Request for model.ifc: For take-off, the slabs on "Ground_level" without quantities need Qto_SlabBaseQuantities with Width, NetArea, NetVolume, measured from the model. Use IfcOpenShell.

First a look at what the model holds.

```python
import ifcopenshell
import ifcopenshell.util.element
import ifcopenshell.util.unit

model = ifcopenshell.open("model.ifc")
print(model.schema)
for unit_type in ("LENGTHUNIT", "AREAUNIT", "VOLUMEUNIT"):
    print(unit_type, ifcopenshell.util.unit.calculate_unit_scale(model, unit_type))
storey = next(s for s in model.by_type("IfcBuildingStorey") if s.Name == "Ground_level")
slabs = [e for e in ifcopenshell.util.element.get_decomposition(storey) if e.is_a("IfcSlab")]
for e in sorted(slabs, key=lambda e: e.id()):
    print(e.id(), e.is_a(), e.Name, list(ifcopenshell.util.element.get_psets(e, qtos_only=True)), sep=" | ")
```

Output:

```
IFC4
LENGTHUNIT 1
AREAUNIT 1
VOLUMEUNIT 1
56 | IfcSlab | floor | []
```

```python
import ifcopenshell
import ifcopenshell.api.pset
import ifcopenshell.geom
import ifcopenshell.util.element
import ifcopenshell.util.shape
import ifcopenshell.util.unit

model = ifcopenshell.open("model.ifc")
unit_scale = ifcopenshell.util.unit.calculate_unit_scale(model)
area_scale = ifcopenshell.util.unit.calculate_unit_scale(model, "AREAUNIT")
volume_scale = ifcopenshell.util.unit.calculate_unit_scale(model, "VOLUMEUNIT")
settings = ifcopenshell.geom.settings()

storey = next(s for s in model.by_type("IfcBuildingStorey") if s.Name == "Ground_level")
slabs = [e for e in ifcopenshell.util.element.get_decomposition(storey) if e.is_a("IfcSlab")]

for e in sorted(slabs, key=lambda e: e.id()):
    if ifcopenshell.util.element.get_psets(e, qtos_only=True, should_inherit=False):
        continue
    # Geometry comes back in metres, in the element's own axes.
    shape = ifcopenshell.geom.create_shape(settings, e)
    values = {
        "Width": ifcopenshell.util.shape.get_z(shape.geometry) / unit_scale,
        "NetArea": ifcopenshell.util.shape.get_footprint_area(shape.geometry) / area_scale,
        "NetVolume": ifcopenshell.util.shape.get_volume(shape.geometry) / volume_scale,
    }
    qto = ifcopenshell.api.pset.add_qto(model, product=e, name="Qto_SlabBaseQuantities")
    ifcopenshell.api.pset.edit_qto(model, qto=qto, properties=values)
    print(e.id(), {k: round(v, 3) for k, v in values.items()})

model.write("model_rev.ifc")
```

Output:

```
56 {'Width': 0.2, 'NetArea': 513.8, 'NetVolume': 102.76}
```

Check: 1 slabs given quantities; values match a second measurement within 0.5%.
